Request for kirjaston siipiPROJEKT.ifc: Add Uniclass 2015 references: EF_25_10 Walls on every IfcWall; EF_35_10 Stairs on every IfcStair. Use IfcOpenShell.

First a look at what the model holds.

```python
import ifcopenshell

model = ifcopenshell.open("kirjaston siipiPROJEKT.ifc")
print(model.schema)
print("classifications:", [c.Name for c in model.by_type("IfcClassification")])
for ifc_class in ("IfcDoor", "IfcRoof", "IfcStair", "IfcWall", "IfcWindow"):
    print(ifc_class, len(model.by_type(ifc_class)))
```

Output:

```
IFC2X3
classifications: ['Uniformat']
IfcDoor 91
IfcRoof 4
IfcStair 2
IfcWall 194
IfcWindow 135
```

```python
import ifcopenshell
import ifcopenshell.api.classification

model = ifcopenshell.open("kirjaston siipiPROJEKT.ifc")

# IFC2X3 requires Source and Edition and has no link from the project to the system.
system = model.create_entity("IfcClassification", Source="NBS", Edition="2015", Name="Uniclass 2015")

codes = {
    "IfcWall": ("EF_25_10", "Walls"),
    "IfcStair": ("EF_35_10", "Stairs"),
}
for ifc_class, (code, name) in codes.items():
    products = model.by_type(ifc_class)
    ifcopenshell.api.classification.add_reference(
        model, products=products, classification=system, identification=code, name=name
    )
    print(code, len(products))

model.write("kirjaston siipiPROJEKT-out.ifc")
```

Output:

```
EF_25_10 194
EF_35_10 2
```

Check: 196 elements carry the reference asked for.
